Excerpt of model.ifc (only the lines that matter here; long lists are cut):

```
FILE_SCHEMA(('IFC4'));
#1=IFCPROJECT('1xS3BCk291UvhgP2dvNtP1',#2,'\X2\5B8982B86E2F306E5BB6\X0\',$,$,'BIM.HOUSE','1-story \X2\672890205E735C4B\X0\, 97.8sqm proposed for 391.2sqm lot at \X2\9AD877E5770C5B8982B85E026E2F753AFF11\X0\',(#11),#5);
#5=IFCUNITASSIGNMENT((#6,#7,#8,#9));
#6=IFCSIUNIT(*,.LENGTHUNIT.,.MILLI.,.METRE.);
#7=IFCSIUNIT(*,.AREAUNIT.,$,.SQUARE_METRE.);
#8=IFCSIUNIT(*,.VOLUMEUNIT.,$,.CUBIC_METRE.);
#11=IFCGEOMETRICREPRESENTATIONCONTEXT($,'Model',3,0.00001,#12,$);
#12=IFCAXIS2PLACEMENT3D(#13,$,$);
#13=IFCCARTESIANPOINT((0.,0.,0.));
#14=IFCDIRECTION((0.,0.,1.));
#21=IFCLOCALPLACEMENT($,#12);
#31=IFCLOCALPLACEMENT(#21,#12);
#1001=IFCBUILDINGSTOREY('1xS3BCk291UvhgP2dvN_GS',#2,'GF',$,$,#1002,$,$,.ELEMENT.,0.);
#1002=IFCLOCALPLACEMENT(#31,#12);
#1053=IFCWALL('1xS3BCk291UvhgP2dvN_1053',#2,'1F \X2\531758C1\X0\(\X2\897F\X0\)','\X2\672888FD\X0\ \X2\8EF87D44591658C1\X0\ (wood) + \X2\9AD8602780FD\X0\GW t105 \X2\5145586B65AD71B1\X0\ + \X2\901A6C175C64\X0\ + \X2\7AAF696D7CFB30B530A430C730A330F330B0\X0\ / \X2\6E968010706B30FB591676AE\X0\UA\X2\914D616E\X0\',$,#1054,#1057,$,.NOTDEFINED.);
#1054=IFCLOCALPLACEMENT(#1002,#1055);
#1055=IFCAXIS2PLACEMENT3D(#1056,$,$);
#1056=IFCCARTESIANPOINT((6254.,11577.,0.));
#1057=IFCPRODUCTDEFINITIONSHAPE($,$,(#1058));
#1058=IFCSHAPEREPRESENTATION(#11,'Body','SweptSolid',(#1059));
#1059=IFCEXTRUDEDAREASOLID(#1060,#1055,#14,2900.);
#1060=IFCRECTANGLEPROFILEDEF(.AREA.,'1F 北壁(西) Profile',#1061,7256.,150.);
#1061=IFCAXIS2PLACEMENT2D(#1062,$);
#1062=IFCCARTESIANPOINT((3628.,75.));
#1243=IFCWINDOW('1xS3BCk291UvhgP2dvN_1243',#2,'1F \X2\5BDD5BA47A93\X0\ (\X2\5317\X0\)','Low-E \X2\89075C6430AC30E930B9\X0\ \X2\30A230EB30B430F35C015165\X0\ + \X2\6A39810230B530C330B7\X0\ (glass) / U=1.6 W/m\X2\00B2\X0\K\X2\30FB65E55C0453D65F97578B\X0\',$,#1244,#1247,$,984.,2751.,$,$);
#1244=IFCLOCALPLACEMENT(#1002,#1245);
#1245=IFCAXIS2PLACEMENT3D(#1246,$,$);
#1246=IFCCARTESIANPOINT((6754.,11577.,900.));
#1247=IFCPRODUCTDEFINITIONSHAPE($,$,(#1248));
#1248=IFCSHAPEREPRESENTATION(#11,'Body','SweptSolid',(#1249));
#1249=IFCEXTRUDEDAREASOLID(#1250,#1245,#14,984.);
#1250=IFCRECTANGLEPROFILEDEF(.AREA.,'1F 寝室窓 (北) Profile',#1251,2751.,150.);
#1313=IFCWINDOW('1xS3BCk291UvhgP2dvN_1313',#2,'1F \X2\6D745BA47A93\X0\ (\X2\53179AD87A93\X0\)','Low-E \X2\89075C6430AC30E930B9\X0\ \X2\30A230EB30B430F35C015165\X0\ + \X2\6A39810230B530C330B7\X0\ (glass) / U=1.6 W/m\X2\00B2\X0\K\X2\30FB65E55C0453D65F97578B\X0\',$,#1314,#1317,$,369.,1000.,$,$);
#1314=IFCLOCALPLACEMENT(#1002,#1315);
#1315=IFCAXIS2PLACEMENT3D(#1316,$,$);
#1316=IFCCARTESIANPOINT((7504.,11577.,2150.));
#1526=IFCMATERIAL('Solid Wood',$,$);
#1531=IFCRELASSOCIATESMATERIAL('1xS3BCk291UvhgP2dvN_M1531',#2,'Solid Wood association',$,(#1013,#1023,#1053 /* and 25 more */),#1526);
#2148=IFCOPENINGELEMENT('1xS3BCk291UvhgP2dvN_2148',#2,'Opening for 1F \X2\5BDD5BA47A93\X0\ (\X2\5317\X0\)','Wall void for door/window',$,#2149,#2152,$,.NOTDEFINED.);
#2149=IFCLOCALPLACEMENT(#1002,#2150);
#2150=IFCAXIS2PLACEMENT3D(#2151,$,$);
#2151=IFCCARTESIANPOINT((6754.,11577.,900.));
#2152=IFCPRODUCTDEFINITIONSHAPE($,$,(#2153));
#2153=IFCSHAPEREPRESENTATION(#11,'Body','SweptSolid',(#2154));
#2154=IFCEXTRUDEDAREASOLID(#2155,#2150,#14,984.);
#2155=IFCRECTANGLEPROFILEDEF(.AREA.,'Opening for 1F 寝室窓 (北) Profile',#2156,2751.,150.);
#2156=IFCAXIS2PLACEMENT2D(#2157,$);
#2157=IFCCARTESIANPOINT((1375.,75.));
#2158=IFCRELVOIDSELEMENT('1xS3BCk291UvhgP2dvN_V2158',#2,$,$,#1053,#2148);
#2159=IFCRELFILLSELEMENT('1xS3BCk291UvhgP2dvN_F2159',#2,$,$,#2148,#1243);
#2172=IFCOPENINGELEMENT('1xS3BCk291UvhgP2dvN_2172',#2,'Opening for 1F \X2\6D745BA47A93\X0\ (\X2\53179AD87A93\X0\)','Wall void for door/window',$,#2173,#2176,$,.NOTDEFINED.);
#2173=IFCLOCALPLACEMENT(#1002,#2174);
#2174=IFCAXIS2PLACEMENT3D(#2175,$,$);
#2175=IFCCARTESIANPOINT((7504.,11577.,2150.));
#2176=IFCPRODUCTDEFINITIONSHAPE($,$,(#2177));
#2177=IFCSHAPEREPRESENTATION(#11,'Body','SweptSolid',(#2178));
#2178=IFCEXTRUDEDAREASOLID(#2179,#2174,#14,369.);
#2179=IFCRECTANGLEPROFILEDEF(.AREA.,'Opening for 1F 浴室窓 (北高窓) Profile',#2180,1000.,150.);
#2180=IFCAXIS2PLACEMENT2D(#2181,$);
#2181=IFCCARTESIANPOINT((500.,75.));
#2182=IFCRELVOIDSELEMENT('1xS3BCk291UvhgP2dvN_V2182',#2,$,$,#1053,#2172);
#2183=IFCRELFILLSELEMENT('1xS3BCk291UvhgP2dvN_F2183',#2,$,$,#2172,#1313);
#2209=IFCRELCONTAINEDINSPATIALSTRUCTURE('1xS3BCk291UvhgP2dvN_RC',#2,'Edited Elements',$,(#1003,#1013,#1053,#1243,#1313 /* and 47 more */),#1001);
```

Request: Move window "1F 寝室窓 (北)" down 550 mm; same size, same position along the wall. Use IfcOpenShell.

```python
import numpy as np
import ifcopenshell
import ifcopenshell.api.geometry
import ifcopenshell.util.placement
import ifcopenshell.util.unit

model = ifcopenshell.open("model.ifc")
unit_scale = ifcopenshell.util.unit.calculate_unit_scale(model)

window = model.by_guid("1xS3BCk291UvhgP2dvN_1243")
opening = window.FillsVoids[0].RelatingOpeningElement
dz = -550.0

shift = np.array([0.0, 0.0, dz])
# The window is not placed relative to its opening, so move both.
for product in (opening, window):
    matrix = ifcopenshell.util.placement.get_local_placement(product.ObjectPlacement)
    matrix[:3, 3] += shift
    ifcopenshell.api.geometry.edit_object_placement(model, product=product, matrix=matrix, is_si=False)

print(f"moved by {dz * unit_scale:+.3f} m")

model.write("model-out.ifc")
```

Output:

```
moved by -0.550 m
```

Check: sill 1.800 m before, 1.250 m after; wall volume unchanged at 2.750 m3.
